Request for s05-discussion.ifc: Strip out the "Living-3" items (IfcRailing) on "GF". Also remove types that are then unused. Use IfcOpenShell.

First a look at what the model holds.

```python
import ifcopenshell
import ifcopenshell.util.element

model = ifcopenshell.open("s05-discussion.ifc")
print(model.schema)
storey = next(s for s in model.by_type("IfcBuildingStorey") if s.Name == "GF")
railings = [e for e in ifcopenshell.util.element.get_decomposition(storey) if e.is_a("IfcRailing")]
seen = {}
for e in railings:
    element_type = ifcopenshell.util.element.get_type(e)
    name = element_type.Name if element_type not in (None, e) else None
    seen[name] = seen.get(name, 0) + 1
for name, count in sorted(seen.items(), key=str):
    print(count, "x", name)
```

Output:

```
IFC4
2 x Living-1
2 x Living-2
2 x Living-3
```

```python
import ifcopenshell
import ifcopenshell.api.root
import ifcopenshell.util.element

model = ifcopenshell.open("s05-discussion.ifc")

storey = next(s for s in model.by_type("IfcBuildingStorey") if s.Name == "GF")
railings = [e for e in ifcopenshell.util.element.get_decomposition(storey) if e.is_a("IfcRailing")]
targets = [e for e in railings if (t := ifcopenshell.util.element.get_type(e)) not in (None, e) and t.Name == "Living-3"]
types = {ifcopenshell.util.element.get_type(e) for e in targets} - {None, *targets}

for e in targets:
    ifcopenshell.api.root.remove_product(model, product=e)
print(len(targets), "removed")

unused = [t for t in types if not ifcopenshell.util.element.get_types(t)]
for t in unused:
    ifcopenshell.api.root.remove_product(model, product=t)
print(len(unused), "unused types removed")

model.write("s05-discussion_edited.ifc")
```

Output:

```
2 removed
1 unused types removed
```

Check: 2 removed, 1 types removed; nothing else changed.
